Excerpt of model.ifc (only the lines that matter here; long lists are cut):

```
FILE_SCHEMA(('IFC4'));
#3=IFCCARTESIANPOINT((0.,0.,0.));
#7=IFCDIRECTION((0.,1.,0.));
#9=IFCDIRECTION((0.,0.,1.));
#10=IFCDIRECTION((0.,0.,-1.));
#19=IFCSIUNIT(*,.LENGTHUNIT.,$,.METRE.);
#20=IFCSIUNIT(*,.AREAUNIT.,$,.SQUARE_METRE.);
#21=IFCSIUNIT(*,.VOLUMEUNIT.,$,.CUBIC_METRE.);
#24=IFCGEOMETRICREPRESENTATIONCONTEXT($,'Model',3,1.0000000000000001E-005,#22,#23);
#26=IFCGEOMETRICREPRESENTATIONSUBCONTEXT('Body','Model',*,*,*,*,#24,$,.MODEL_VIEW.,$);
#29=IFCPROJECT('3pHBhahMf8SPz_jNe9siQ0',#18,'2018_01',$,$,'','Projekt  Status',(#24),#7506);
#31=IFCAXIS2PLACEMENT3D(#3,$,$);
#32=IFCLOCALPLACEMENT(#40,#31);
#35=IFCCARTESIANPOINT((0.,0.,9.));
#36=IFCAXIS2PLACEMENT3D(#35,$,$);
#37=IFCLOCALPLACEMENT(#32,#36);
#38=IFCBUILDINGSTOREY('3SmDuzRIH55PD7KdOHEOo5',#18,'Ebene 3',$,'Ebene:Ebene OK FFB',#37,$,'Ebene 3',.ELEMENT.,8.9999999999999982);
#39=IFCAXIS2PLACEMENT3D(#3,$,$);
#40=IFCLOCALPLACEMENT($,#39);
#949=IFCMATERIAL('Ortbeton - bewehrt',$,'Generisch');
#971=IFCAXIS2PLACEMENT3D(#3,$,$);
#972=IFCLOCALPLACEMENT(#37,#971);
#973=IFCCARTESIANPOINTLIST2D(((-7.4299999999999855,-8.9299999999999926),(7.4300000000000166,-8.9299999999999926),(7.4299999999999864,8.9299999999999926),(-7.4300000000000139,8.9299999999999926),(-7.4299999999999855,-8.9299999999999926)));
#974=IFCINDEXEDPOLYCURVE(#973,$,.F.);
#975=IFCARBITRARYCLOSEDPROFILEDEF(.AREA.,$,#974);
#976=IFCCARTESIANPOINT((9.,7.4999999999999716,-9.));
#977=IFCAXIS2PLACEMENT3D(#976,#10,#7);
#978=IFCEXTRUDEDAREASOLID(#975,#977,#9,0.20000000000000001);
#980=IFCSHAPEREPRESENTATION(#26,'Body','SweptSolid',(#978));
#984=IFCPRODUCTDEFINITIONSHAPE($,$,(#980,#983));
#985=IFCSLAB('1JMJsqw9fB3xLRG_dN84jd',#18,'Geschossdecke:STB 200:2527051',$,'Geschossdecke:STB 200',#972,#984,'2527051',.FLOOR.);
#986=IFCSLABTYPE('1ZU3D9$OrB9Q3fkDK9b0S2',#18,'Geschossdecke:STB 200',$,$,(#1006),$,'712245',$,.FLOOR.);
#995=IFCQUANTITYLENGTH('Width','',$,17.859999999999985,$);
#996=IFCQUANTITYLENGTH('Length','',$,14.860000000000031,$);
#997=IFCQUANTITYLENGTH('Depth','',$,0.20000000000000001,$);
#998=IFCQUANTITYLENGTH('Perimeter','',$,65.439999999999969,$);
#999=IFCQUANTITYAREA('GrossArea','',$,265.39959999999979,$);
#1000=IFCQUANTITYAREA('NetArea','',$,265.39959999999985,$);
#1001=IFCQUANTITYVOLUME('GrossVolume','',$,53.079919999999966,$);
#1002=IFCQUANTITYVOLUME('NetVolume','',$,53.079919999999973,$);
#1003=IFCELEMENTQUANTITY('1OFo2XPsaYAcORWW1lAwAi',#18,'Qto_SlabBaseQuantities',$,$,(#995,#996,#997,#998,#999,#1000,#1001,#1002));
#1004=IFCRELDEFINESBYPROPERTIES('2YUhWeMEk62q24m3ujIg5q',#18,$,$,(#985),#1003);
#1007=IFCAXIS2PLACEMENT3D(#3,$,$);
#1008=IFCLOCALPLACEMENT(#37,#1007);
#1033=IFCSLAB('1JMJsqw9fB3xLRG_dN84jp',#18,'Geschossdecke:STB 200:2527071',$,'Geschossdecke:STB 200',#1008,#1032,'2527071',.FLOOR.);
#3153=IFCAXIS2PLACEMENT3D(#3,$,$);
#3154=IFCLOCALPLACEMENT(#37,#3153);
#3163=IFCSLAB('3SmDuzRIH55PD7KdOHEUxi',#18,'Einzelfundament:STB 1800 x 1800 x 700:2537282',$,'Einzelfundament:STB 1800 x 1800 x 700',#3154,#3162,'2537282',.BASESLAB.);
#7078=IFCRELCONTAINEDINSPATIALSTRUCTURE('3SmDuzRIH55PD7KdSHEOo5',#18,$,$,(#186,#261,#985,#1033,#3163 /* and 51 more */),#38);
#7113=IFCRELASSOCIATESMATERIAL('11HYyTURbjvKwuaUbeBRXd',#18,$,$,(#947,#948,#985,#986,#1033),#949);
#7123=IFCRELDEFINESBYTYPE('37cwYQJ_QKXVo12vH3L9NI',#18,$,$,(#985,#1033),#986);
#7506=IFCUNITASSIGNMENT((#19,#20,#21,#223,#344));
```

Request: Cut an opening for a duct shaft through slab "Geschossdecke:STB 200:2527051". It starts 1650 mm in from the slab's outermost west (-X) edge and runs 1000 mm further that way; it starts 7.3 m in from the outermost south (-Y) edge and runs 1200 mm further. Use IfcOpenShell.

```python
import numpy as np
import ifcopenshell
import ifcopenshell.api.feature
import ifcopenshell.api.geometry
import ifcopenshell.api.pset
import ifcopenshell.api.root
import ifcopenshell.geom
import ifcopenshell.util.element
import ifcopenshell.util.placement
import ifcopenshell.util.representation
import ifcopenshell.util.shape
import ifcopenshell.util.unit

model = ifcopenshell.open("model.ifc")
unit_scale = ifcopenshell.util.unit.calculate_unit_scale(model)
area_scale = ifcopenshell.util.unit.calculate_unit_scale(model, "AREAUNIT")
volume_scale = ifcopenshell.util.unit.calculate_unit_scale(model, "VOLUMEUNIT")
settings = ifcopenshell.geom.settings()


def volume(element):
    """Net volume in cubic metres, openings subtracted."""
    shape = ifcopenshell.geom.create_shape(settings, element)
    return ifcopenshell.util.shape.get_volume(shape.geometry)


slab = model.by_guid("1JMJsqw9fB3xLRG_dN84jd")
before = volume(slab)

# Extent in the slab's own axes, in metres. The edges named are its -X and -Y sides.
slab_shape = ifcopenshell.geom.create_shape(settings, slab)
vertices = ifcopenshell.util.shape.get_vertices(slab_shape.geometry)
x_min, y_min, bottom = vertices.min(axis=0)
top = vertices[:, 2].max()

opening = ifcopenshell.api.root.create_entity(model, ifc_class="IfcOpeningElement", name="Duct shaft opening", predefined_type="OPENING")
context = ifcopenshell.util.representation.get_context(model, "Model", "Body", "MODEL_VIEW")
width, depth = 1, 1.2
outline = [(0.0, 0.0), (width, 0.0), (width, depth), (0.0, depth), (0.0, 0.0)]
# Overshoot both faces by 50 mm so the cut is clean.
shape = ifcopenshell.api.geometry.add_slab_representation(
    model, context=context, depth=top - bottom + 0.1, polyline=outline
)
ifcopenshell.api.geometry.assign_representation(model, product=opening, representation=shape)

matrix = ifcopenshell.util.placement.get_local_placement(slab.ObjectPlacement)
matrix[:, 3] = matrix @ np.append(np.array([x_min + 1.65, y_min + 7.3, bottom - 0.05]) / unit_scale, 1.0)
ifcopenshell.api.geometry.edit_object_placement(model, product=opening, matrix=matrix, is_si=False)
ifcopenshell.api.feature.add_feature(model, feature=opening, element=slab)

after = volume(slab)

# Update the slab's stored quantities.
qto = model.by_id(ifcopenshell.util.element.get_pset(slab, "Qto_SlabBaseQuantities", should_inherit=False)["id"])
ifcopenshell.api.pset.edit_qto(model, qto=qto, properties={
    "NetArea": after / (top - bottom) / area_scale,
    "NetVolume": after / volume_scale,
})

print(f"slab volume {before:.3f} -> {after:.3f} m3")

model.write("model_updated.ifc")
```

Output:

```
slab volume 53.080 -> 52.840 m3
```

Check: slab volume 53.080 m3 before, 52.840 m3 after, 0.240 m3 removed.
